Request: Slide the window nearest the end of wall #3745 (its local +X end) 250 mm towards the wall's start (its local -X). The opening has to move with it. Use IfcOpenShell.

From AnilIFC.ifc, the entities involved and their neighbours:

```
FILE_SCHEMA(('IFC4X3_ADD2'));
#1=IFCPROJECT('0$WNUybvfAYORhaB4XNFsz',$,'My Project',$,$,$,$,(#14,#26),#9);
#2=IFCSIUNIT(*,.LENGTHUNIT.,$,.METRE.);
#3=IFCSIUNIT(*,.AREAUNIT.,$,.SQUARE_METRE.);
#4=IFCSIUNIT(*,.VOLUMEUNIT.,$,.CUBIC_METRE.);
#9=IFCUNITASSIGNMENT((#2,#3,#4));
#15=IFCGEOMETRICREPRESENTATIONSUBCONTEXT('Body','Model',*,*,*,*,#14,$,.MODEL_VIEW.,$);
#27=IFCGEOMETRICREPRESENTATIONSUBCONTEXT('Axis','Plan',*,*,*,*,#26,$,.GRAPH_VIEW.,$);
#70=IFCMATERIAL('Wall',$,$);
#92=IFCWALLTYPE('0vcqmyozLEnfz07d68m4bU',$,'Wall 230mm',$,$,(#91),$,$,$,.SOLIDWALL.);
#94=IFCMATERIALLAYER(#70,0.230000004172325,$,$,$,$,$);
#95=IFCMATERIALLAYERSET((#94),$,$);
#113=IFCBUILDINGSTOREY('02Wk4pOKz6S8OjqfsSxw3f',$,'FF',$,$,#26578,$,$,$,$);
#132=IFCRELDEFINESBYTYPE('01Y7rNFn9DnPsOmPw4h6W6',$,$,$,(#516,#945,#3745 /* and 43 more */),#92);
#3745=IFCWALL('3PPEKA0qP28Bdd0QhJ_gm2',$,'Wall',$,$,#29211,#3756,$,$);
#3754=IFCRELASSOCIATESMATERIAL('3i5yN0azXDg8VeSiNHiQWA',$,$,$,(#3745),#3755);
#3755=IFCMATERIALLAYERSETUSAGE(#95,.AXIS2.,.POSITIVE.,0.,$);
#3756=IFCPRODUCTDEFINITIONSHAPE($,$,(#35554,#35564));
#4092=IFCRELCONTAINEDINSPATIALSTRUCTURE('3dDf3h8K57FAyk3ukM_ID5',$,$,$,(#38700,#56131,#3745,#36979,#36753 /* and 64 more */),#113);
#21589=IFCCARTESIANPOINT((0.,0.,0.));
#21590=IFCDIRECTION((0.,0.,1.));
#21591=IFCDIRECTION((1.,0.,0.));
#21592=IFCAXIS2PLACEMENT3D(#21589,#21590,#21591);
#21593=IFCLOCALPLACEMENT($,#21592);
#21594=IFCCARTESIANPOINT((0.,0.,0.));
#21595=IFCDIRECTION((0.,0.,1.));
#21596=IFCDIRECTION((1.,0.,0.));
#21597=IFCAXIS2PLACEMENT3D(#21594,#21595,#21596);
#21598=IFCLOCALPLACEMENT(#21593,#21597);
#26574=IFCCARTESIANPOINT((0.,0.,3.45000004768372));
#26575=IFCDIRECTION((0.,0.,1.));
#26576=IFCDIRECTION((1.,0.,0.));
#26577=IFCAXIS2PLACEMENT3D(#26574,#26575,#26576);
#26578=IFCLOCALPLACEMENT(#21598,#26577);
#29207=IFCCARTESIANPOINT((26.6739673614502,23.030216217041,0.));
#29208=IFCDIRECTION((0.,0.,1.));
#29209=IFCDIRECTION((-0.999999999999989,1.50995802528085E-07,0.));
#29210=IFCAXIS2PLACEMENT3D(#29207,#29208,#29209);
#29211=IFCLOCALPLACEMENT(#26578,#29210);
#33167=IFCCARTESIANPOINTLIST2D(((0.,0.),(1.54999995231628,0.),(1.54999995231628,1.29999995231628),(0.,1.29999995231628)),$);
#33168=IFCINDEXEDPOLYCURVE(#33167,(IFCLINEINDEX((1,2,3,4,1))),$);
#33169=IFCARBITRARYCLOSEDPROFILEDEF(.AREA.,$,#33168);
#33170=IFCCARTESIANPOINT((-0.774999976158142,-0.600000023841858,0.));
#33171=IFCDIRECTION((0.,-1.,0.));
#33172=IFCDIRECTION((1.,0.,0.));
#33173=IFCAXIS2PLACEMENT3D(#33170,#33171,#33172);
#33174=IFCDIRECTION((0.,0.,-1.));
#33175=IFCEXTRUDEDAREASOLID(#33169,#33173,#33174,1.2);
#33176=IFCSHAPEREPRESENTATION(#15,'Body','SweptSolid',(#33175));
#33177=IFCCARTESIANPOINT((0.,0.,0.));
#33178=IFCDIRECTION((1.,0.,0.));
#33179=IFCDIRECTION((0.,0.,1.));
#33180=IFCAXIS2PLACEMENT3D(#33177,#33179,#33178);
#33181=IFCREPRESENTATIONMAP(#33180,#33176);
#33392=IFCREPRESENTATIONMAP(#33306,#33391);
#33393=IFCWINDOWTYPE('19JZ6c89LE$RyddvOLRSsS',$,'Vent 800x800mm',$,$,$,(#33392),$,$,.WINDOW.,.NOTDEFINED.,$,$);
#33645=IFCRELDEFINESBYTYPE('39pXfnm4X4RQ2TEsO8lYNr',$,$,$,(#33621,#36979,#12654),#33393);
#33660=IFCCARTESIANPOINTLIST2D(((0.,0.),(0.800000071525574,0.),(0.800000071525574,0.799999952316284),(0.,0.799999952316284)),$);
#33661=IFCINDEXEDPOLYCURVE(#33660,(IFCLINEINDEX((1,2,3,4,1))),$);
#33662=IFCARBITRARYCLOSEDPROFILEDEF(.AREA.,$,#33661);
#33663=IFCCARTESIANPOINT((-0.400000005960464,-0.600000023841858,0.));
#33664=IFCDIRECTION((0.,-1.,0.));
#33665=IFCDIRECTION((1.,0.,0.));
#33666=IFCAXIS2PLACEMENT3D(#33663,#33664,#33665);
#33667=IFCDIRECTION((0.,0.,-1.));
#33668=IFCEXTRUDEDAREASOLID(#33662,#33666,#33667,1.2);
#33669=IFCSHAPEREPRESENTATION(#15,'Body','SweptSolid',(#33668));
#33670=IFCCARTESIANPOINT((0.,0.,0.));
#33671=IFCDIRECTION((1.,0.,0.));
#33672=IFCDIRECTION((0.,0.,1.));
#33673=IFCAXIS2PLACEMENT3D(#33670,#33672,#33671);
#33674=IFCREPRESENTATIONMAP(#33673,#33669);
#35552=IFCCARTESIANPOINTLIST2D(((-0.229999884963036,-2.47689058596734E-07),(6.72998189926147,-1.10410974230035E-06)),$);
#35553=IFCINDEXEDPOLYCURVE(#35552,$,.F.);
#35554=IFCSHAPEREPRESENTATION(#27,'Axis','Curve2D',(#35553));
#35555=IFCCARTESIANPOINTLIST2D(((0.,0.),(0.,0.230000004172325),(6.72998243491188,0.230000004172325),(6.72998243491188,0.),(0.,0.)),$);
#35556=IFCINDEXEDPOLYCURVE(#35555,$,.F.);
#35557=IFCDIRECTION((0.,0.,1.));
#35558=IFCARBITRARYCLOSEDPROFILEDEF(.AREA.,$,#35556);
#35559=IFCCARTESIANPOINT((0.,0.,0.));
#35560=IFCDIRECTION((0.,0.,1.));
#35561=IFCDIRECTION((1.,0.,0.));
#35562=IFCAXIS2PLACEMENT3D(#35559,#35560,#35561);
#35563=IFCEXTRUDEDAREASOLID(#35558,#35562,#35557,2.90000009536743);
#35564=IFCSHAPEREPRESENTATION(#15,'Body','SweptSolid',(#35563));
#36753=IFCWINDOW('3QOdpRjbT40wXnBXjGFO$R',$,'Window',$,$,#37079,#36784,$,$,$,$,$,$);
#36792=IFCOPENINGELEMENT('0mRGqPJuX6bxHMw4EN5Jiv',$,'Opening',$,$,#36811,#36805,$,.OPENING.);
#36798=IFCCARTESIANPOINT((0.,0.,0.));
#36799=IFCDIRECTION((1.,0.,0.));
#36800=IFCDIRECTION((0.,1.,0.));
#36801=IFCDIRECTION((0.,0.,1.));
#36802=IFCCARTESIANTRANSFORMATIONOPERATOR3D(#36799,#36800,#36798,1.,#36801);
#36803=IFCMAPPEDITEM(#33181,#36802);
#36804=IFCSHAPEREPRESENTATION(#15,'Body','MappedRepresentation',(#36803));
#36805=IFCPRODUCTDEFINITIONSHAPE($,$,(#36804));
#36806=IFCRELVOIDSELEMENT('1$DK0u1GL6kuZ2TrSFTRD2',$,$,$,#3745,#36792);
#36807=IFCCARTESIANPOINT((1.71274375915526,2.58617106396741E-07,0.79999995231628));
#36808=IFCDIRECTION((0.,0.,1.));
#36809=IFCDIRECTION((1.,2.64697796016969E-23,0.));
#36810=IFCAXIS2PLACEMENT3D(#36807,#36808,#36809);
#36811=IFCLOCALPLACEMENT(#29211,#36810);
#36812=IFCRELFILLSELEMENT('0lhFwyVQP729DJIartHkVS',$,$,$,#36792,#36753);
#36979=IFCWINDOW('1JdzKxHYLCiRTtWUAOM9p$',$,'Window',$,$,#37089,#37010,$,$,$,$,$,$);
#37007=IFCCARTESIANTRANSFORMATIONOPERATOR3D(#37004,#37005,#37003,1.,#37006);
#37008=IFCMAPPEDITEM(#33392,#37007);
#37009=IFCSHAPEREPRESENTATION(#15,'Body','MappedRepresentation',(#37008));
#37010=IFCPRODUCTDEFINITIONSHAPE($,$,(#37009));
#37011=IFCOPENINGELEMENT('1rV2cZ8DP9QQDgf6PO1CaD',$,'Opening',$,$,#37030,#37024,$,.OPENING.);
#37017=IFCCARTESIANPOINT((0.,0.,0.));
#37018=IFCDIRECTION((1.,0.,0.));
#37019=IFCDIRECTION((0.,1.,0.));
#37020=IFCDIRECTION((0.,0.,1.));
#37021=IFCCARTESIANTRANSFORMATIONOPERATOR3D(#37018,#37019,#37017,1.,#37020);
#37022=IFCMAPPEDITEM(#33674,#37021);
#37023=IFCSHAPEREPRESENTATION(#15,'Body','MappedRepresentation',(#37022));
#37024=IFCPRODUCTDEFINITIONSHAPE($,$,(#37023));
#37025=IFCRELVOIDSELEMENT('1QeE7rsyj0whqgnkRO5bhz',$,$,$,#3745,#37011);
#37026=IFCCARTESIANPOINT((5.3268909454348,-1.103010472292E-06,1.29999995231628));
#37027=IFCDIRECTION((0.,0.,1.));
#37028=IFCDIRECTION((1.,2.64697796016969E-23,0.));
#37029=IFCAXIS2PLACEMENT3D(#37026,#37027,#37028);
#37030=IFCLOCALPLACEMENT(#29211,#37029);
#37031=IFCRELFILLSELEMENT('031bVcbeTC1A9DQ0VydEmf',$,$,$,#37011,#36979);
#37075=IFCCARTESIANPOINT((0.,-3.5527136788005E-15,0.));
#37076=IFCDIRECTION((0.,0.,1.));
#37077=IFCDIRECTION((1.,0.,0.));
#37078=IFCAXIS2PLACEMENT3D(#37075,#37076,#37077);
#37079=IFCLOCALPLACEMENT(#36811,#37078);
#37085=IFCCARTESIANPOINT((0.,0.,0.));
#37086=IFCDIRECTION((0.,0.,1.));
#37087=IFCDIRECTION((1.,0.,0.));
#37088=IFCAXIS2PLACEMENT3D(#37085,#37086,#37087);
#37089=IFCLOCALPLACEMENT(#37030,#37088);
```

```python
import ifcopenshell
import ifcopenshell.api.geometry
import ifcopenshell.util.placement
import ifcopenshell.util.unit

model = ifcopenshell.open("AnilIFC.ifc")
unit_scale = ifcopenshell.util.unit.calculate_unit_scale(model)

window = model.by_id(36979)
opening = window.FillsVoids[0].RelatingOpeningElement
wall = opening.VoidsElements[0].RelatingBuildingElement

wall_matrix = ifcopenshell.util.placement.get_local_placement(wall.ObjectPlacement)
shift = wall_matrix[:3, 0] * -0.25 / unit_scale
before = ifcopenshell.util.placement.get_local_placement(window.ObjectPlacement)[:3, 3].copy()

# The window is placed relative to its opening, so it follows when the opening moves.
matrix = ifcopenshell.util.placement.get_local_placement(opening.ObjectPlacement)
matrix[:3, 3] += shift
ifcopenshell.api.geometry.edit_object_placement(
    model, product=opening, matrix=matrix, is_si=False, should_transform_children=True
)

after = ifcopenshell.util.placement.get_local_placement(window.ObjectPlacement)[:3, 3]
print("window moved by", (after - before).round(3) + 0.0)

model.write("AnilIFC-out.ifc")
```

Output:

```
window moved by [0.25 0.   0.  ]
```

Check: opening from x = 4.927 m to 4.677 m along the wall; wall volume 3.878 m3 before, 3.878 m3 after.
